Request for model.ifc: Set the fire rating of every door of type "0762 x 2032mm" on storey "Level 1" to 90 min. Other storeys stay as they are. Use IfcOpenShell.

First a look at what the model holds.

```python
import ifcopenshell
import ifcopenshell.util.element

model = ifcopenshell.open("model.ifc")
print(model.schema)
storey = next(s for s in model.by_type("IfcBuildingStorey") if s.Name == "Level 1")
doors = [e for e in ifcopenshell.util.element.get_decomposition(storey) if e.is_a("IfcDoor")]
seen = {}
for e in doors:
    element_type = ifcopenshell.util.element.get_type(e)
    key = (element_type.Name if element_type != e and element_type else None, ifcopenshell.util.element.get_pset(e, "Pset_DoorCommon", "FireRating"))
    seen[key] = seen.get(key, 0) + 1
for (name, value), count in sorted(seen.items(), key=str):
    print(count, "x", name, "|", value)
```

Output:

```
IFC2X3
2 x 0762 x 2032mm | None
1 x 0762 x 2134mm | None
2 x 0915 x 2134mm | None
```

```python
import ifcopenshell
import ifcopenshell.api.pset
import ifcopenshell.util.element

model = ifcopenshell.open("model.ifc")

storey = next(s for s in model.by_type("IfcBuildingStorey") if s.Name == "Level 1")
doors = [e for e in ifcopenshell.util.element.get_decomposition(storey) if e.is_a("IfcDoor")]

count = 0
for e in doors:
    element_type = ifcopenshell.util.element.get_type(e)
    if element_type in (None, e) or element_type.Name != "0762 x 2032mm":
        continue
    # add_pset returns the element's existing set when there is one.
    pset = ifcopenshell.api.pset.add_pset(model, product=e, name="Pset_DoorCommon")
    ifcopenshell.api.pset.edit_pset(model, pset=pset, properties={"FireRating": "90 min"})
    count += 1

print(count, "doors updated")

model.write("model-out.ifc")
```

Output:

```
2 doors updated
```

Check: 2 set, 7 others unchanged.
